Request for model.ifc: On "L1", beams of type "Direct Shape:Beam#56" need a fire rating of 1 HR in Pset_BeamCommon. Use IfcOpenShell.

First a look at what the model holds.

```python
import ifcopenshell
import ifcopenshell.util.element

model = ifcopenshell.open("model.ifc")
print(model.schema)
storey = next(s for s in model.by_type("IfcBuildingStorey") if s.Name == "L1")
beams = [e for e in ifcopenshell.util.element.get_decomposition(storey) if e.is_a("IfcBeam")]
seen = {}
for e in beams:
    element_type = ifcopenshell.util.element.get_type(e)
    key = (element_type.Name if element_type != e and element_type else None, ifcopenshell.util.element.get_pset(e, "Pset_BeamCommon", "FireRating"))
    seen[key] = seen.get(key, 0) + 1
for (name, value), count in sorted(seen.items(), key=str):
    print(count, "x", name, "|", value)
```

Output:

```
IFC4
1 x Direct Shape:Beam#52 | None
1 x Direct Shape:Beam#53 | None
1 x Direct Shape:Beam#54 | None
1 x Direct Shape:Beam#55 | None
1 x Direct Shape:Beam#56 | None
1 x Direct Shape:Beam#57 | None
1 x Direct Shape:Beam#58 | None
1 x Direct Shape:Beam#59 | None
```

```python
import ifcopenshell
import ifcopenshell.api.pset
import ifcopenshell.util.element

model = ifcopenshell.open("model.ifc")

storey = next(s for s in model.by_type("IfcBuildingStorey") if s.Name == "L1")
beams = [e for e in ifcopenshell.util.element.get_decomposition(storey) if e.is_a("IfcBeam")]

count = 0
for e in beams:
    element_type = ifcopenshell.util.element.get_type(e)
    if element_type in (None, e) or element_type.Name != "Direct Shape:Beam#56":
        continue
    # add_pset returns the element's existing set when there is one.
    pset = ifcopenshell.api.pset.add_pset(model, product=e, name="Pset_BeamCommon")
    ifcopenshell.api.pset.edit_pset(model, pset=pset, properties={"FireRating": "1 HR"})
    count += 1

print(count, "beams updated")

model.write("model_rev.ifc")
```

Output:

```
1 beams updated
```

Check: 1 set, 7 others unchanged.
